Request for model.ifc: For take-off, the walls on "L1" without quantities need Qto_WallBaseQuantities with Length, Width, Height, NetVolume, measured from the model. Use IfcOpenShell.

First a look at what the model holds.

```python
import ifcopenshell
import ifcopenshell.util.element
import ifcopenshell.util.unit

model = ifcopenshell.open("model.ifc")
print(model.schema)
for unit_type in ("LENGTHUNIT", "AREAUNIT", "VOLUMEUNIT"):
    print(unit_type, ifcopenshell.util.unit.calculate_unit_scale(model, unit_type))
storey = next(s for s in model.by_type("IfcBuildingStorey") if s.Name == "L1")
walls = [e for e in ifcopenshell.util.element.get_decomposition(storey) if e.is_a("IfcWall")]
for e in sorted(walls, key=lambda e: e.id()):
    print(e.id(), e.is_a(), e.Name, list(ifcopenshell.util.element.get_psets(e, qtos_only=True)), sep=" | ")
```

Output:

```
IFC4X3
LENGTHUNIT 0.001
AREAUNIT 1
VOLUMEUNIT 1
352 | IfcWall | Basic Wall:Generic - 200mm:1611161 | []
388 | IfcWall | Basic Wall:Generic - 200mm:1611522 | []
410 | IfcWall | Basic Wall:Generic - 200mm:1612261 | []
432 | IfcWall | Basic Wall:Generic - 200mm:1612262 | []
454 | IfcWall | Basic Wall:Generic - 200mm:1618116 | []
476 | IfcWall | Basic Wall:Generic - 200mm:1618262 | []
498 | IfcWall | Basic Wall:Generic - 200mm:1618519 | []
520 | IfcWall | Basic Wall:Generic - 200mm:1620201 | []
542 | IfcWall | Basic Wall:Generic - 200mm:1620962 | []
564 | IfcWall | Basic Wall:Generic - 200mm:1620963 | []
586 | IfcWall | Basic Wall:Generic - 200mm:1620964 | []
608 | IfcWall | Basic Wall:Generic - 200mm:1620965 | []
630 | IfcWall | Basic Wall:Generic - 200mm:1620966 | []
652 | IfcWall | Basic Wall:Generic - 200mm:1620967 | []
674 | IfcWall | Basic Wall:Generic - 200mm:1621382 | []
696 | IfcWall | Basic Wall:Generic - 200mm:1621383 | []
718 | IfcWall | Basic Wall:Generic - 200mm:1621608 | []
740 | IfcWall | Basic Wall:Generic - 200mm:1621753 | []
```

```python
import ifcopenshell
import ifcopenshell.api.pset
import ifcopenshell.geom
import ifcopenshell.util.element
import ifcopenshell.util.shape
import ifcopenshell.util.unit

model = ifcopenshell.open("model.ifc")
unit_scale = ifcopenshell.util.unit.calculate_unit_scale(model)
volume_scale = ifcopenshell.util.unit.calculate_unit_scale(model, "VOLUMEUNIT")
settings = ifcopenshell.geom.settings()

storey = next(s for s in model.by_type("IfcBuildingStorey") if s.Name == "L1")
walls = [e for e in ifcopenshell.util.element.get_decomposition(storey) if e.is_a("IfcWall")]

for e in sorted(walls, key=lambda e: e.id()):
    if ifcopenshell.util.element.get_psets(e, qtos_only=True, should_inherit=False):
        continue
    # Geometry comes back in metres, in the element's own axes.
    shape = ifcopenshell.geom.create_shape(settings, e)
    values = {
        "Length": ifcopenshell.util.shape.get_x(shape.geometry) / unit_scale,
        "Width": ifcopenshell.util.shape.get_y(shape.geometry) / unit_scale,
        "Height": ifcopenshell.util.shape.get_z(shape.geometry) / unit_scale,
        "NetVolume": ifcopenshell.util.shape.get_volume(shape.geometry) / volume_scale,
    }
    qto = ifcopenshell.api.pset.add_qto(model, product=e, name="Qto_WallBaseQuantities")
    ifcopenshell.api.pset.edit_qto(model, qto=qto, properties=values)
    print(e.id(), {k: round(v, 3) for k, v in values.items()})

model.write("model_updated.ifc")
```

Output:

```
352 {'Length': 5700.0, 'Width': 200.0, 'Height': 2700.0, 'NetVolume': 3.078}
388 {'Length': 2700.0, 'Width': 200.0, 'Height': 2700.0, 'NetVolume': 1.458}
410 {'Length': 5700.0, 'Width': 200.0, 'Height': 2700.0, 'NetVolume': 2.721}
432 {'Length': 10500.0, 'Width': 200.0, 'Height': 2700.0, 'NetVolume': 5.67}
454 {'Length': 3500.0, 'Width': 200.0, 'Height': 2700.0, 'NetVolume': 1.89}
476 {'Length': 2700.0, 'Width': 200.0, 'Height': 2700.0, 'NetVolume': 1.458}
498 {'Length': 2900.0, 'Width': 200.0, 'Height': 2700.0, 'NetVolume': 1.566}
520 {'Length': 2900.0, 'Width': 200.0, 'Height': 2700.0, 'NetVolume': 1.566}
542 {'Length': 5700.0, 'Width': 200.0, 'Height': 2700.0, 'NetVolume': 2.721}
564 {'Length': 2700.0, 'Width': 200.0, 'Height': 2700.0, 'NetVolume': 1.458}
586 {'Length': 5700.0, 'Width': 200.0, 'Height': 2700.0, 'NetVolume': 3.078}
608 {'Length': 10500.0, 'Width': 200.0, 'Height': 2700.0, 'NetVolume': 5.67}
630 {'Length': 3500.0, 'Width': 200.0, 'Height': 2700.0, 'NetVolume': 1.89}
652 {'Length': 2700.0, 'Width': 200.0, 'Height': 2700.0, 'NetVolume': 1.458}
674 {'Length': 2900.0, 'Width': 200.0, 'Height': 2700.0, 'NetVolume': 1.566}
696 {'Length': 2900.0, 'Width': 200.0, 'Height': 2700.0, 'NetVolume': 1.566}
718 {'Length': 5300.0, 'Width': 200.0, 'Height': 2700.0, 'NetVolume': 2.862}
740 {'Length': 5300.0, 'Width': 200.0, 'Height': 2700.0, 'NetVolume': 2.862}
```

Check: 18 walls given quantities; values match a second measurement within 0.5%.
